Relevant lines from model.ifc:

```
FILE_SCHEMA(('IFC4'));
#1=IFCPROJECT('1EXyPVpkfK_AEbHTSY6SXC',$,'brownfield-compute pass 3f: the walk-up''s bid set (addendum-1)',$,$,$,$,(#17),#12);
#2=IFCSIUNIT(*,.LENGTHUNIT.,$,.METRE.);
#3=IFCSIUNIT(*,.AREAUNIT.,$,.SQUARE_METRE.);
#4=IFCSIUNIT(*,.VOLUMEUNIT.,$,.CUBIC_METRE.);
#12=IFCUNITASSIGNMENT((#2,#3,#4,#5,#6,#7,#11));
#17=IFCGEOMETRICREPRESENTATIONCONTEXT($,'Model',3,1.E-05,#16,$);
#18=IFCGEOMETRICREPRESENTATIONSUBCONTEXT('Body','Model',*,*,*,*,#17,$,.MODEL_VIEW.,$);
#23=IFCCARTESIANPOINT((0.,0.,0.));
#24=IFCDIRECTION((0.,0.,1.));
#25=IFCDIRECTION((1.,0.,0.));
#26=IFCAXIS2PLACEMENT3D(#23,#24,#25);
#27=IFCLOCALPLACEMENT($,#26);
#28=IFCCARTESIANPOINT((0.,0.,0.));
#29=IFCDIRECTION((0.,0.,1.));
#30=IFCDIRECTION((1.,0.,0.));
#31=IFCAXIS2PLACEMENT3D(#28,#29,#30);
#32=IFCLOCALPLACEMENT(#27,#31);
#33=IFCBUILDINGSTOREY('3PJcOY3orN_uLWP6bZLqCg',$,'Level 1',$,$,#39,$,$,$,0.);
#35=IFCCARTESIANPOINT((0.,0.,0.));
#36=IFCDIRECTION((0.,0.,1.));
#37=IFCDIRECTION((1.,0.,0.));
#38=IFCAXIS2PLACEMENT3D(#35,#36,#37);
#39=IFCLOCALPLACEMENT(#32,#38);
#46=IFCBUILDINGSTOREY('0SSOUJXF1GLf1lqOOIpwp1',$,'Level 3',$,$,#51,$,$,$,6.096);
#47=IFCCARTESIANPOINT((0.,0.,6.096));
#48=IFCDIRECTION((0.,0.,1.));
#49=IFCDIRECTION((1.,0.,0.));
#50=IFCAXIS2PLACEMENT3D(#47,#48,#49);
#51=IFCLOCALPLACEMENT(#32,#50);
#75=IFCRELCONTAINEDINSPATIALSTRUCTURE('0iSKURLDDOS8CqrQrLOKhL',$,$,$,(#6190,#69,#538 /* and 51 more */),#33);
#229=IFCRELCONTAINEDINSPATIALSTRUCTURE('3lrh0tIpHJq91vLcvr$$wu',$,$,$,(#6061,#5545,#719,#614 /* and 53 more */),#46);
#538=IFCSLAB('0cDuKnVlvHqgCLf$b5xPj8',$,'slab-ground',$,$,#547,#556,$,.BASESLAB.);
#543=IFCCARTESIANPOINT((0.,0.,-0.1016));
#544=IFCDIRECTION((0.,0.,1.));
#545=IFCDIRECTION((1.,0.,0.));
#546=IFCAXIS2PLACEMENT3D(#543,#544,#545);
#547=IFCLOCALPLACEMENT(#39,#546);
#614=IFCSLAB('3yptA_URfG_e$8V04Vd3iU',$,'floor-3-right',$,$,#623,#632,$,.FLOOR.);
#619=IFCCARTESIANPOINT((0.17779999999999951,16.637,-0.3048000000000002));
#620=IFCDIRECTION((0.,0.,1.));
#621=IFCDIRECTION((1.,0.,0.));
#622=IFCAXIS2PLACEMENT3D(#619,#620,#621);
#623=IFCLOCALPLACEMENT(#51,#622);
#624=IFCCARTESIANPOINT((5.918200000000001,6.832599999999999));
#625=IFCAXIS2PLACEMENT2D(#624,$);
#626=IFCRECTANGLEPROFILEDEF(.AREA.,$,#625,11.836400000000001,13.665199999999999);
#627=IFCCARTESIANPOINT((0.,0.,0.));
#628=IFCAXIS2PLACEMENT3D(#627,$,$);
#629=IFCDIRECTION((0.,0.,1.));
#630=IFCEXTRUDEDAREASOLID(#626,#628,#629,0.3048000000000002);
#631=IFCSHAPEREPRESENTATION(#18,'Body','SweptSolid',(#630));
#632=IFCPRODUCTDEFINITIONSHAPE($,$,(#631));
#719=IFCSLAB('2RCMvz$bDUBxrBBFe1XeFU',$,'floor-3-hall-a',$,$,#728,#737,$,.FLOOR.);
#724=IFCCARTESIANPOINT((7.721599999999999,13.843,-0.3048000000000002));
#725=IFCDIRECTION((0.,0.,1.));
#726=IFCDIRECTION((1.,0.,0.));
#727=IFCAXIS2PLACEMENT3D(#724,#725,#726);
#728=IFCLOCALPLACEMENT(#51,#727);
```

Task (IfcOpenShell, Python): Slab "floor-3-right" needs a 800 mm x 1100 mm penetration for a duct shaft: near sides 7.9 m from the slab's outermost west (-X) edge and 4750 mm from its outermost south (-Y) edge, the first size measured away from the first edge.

```python
import numpy as np
import ifcopenshell
import ifcopenshell.api.feature
import ifcopenshell.api.geometry
import ifcopenshell.api.root
import ifcopenshell.geom
import ifcopenshell.util.placement
import ifcopenshell.util.representation
import ifcopenshell.util.shape
import ifcopenshell.util.unit

model = ifcopenshell.open("model.ifc")
unit_scale = ifcopenshell.util.unit.calculate_unit_scale(model)
settings = ifcopenshell.geom.settings()


def volume(element):
    """Net volume in cubic metres, openings subtracted."""
    shape = ifcopenshell.geom.create_shape(settings, element)
    return ifcopenshell.util.shape.get_volume(shape.geometry)


slab = model.by_id(614)
before = volume(slab)

# Extent in the slab's own axes, in metres. The edges named are its -X and -Y sides.
slab_shape = ifcopenshell.geom.create_shape(settings, slab)
vertices = ifcopenshell.util.shape.get_vertices(slab_shape.geometry)
x_min, y_min, bottom = vertices.min(axis=0)
top = vertices[:, 2].max()

opening = ifcopenshell.api.root.create_entity(model, ifc_class="IfcOpeningElement", name="Duct shaft opening", predefined_type="OPENING")
context = ifcopenshell.util.representation.get_context(model, "Model", "Body", "MODEL_VIEW")
width, depth = 0.8, 1.1
outline = [(0.0, 0.0), (width, 0.0), (width, depth), (0.0, depth), (0.0, 0.0)]
# Overshoot both faces by 50 mm so the cut is clean.
shape = ifcopenshell.api.geometry.add_slab_representation(
    model, context=context, depth=top - bottom + 0.1, polyline=outline
)
ifcopenshell.api.geometry.assign_representation(model, product=opening, representation=shape)

matrix = ifcopenshell.util.placement.get_local_placement(slab.ObjectPlacement)
matrix[:, 3] = matrix @ np.append(np.array([x_min + 7.9, y_min + 4.75, bottom - 0.05]) / unit_scale, 1.0)
ifcopenshell.api.geometry.edit_object_placement(model, product=opening, matrix=matrix, is_si=False)
ifcopenshell.api.feature.add_feature(model, feature=opening, element=slab)

after = volume(slab)

print(f"slab volume {before:.3f} -> {after:.3f} m3")

model.write("model_updated.ifc")
```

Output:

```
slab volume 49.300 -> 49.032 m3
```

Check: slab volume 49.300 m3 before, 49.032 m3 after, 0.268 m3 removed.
